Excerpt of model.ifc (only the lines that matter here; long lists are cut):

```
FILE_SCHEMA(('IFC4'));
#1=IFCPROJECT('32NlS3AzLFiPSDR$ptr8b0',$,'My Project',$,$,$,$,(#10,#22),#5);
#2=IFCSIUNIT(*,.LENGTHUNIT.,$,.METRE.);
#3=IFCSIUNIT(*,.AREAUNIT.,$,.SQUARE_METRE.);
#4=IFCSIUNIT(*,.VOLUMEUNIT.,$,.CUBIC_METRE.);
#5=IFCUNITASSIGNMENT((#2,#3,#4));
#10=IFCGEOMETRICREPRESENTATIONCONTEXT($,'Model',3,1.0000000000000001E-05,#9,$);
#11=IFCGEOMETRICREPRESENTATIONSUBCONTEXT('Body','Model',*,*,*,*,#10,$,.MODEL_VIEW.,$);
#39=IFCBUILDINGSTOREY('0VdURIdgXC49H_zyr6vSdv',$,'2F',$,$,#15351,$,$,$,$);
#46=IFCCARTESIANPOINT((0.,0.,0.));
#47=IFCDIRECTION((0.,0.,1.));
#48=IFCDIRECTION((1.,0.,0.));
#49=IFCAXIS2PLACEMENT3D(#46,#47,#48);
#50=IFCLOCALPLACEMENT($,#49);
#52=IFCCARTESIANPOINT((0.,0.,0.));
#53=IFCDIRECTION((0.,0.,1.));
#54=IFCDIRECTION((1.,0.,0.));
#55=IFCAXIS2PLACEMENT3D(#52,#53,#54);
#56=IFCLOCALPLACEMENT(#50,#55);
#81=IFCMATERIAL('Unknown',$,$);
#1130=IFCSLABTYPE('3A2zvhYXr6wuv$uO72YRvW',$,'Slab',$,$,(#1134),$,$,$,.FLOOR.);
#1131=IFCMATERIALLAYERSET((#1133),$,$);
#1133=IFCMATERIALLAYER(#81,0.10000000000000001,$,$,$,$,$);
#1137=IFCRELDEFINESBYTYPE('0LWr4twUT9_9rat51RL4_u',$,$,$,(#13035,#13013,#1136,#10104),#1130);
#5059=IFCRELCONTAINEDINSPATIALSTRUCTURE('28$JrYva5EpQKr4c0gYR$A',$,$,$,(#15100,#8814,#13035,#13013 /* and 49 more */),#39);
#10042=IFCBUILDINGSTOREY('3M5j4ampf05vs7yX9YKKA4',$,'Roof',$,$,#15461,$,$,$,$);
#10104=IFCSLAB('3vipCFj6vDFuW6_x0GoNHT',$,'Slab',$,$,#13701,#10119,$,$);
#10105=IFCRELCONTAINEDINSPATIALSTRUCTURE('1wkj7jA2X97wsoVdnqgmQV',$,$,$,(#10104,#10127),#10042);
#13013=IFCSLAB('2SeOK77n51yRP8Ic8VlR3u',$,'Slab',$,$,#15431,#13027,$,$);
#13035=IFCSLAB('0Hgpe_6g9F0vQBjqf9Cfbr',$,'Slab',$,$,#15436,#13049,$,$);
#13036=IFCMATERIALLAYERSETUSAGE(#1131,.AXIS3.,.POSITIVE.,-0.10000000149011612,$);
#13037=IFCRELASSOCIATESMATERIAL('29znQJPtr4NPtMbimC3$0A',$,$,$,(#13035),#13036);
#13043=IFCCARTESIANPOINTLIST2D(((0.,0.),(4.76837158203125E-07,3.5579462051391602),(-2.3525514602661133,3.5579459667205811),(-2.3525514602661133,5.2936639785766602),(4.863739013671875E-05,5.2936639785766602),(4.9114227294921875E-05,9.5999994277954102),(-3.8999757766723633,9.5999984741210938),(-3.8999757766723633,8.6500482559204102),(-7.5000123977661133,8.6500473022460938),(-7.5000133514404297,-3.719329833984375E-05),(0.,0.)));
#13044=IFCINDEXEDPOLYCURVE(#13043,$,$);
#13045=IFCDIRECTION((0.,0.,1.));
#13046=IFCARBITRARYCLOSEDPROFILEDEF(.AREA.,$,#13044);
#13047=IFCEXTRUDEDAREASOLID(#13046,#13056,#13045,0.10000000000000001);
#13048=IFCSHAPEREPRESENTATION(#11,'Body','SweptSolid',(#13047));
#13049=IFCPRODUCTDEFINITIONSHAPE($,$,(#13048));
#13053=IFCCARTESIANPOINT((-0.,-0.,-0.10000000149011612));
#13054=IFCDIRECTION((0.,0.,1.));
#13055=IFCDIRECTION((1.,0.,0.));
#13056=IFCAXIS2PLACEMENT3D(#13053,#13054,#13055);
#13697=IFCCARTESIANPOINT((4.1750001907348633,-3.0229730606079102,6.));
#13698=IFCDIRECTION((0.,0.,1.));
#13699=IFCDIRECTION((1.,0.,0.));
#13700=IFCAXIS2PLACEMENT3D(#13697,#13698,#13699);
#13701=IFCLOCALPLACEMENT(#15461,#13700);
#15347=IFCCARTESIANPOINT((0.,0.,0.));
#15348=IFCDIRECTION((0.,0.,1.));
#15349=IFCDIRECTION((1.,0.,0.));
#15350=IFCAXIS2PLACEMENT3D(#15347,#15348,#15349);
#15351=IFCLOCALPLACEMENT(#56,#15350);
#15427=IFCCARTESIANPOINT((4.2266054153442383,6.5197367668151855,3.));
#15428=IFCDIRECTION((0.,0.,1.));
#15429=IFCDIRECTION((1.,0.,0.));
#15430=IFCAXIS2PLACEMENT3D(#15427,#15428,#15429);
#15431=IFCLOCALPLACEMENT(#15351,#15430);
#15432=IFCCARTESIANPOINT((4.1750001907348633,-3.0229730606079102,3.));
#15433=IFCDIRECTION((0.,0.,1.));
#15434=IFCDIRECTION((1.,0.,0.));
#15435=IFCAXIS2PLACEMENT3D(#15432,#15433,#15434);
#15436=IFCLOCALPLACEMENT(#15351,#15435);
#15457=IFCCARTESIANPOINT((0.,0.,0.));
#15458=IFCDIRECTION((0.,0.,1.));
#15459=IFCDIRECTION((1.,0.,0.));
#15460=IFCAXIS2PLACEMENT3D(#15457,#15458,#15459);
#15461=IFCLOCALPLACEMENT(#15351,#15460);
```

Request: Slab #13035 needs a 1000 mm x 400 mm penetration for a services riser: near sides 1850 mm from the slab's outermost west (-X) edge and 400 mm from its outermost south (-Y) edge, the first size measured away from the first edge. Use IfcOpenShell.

```python
import numpy as np
import ifcopenshell
import ifcopenshell.api.feature
import ifcopenshell.api.geometry
import ifcopenshell.api.root
import ifcopenshell.geom
import ifcopenshell.util.placement
import ifcopenshell.util.representation
import ifcopenshell.util.shape
import ifcopenshell.util.unit

model = ifcopenshell.open("model.ifc")
unit_scale = ifcopenshell.util.unit.calculate_unit_scale(model)
settings = ifcopenshell.geom.settings()


def volume(element):
    """Net volume in cubic metres, openings subtracted."""
    shape = ifcopenshell.geom.create_shape(settings, element)
    return ifcopenshell.util.shape.get_volume(shape.geometry)


slab = model.by_id(13035)
before = volume(slab)

# Extent in the slab's own axes, in metres. The edges named are its -X and -Y sides.
slab_shape = ifcopenshell.geom.create_shape(settings, slab)
vertices = ifcopenshell.util.shape.get_vertices(slab_shape.geometry)
x_min, y_min, bottom = vertices.min(axis=0)
top = vertices[:, 2].max()

opening = ifcopenshell.api.root.create_entity(model, ifc_class="IfcOpeningElement", name="Services riser opening", predefined_type="OPENING")
context = ifcopenshell.util.representation.get_context(model, "Model", "Body", "MODEL_VIEW")
width, depth = 1, 0.4
outline = [(0.0, 0.0), (width, 0.0), (width, depth), (0.0, depth), (0.0, 0.0)]
# Overshoot both faces by 50 mm so the cut is clean.
shape = ifcopenshell.api.geometry.add_slab_representation(
    model, context=context, depth=top - bottom + 0.1, polyline=outline
)
ifcopenshell.api.geometry.assign_representation(model, product=opening, representation=shape)

matrix = ifcopenshell.util.placement.get_local_placement(slab.ObjectPlacement)
matrix[:, 3] = matrix @ np.append(np.array([x_min + 1.85, y_min + 0.4, bottom - 0.05]) / unit_scale, 1.0)
ifcopenshell.api.geometry.edit_object_placement(model, product=opening, matrix=matrix, is_si=False)
ifcopenshell.api.feature.add_feature(model, feature=opening, element=slab)

after = volume(slab)

print(f"slab volume {before:.3f} -> {after:.3f} m3")

model.write("model_updated.ifc")
```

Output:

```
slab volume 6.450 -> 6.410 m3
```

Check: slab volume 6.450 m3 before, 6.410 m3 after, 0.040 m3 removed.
